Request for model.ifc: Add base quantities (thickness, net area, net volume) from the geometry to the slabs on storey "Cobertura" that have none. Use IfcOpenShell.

First a look at what the model holds.

```python
import ifcopenshell
import ifcopenshell.util.element
import ifcopenshell.util.unit

model = ifcopenshell.open("model.ifc")
print(model.schema)
for unit_type in ("LENGTHUNIT", "AREAUNIT", "VOLUMEUNIT"):
    print(unit_type, ifcopenshell.util.unit.calculate_unit_scale(model, unit_type))
storey = next(s for s in model.by_type("IfcBuildingStorey") if s.Name == "Cobertura")
slabs = [e for e in ifcopenshell.util.element.get_decomposition(storey) if e.is_a("IfcSlab")]
for e in sorted(slabs, key=lambda e: e.id()):
    print(e.id(), e.is_a(), e.Name, list(ifcopenshell.util.element.get_psets(e, qtos_only=True)), sep=" | ")
```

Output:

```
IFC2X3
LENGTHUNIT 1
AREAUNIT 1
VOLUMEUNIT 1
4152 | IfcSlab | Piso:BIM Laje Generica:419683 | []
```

```python
import ifcopenshell
import ifcopenshell.api.pset
import ifcopenshell.geom
import ifcopenshell.util.element
import ifcopenshell.util.shape
import ifcopenshell.util.unit

model = ifcopenshell.open("model.ifc")
unit_scale = ifcopenshell.util.unit.calculate_unit_scale(model)
area_scale = ifcopenshell.util.unit.calculate_unit_scale(model, "AREAUNIT")
volume_scale = ifcopenshell.util.unit.calculate_unit_scale(model, "VOLUMEUNIT")
settings = ifcopenshell.geom.settings()

storey = next(s for s in model.by_type("IfcBuildingStorey") if s.Name == "Cobertura")
slabs = [e for e in ifcopenshell.util.element.get_decomposition(storey) if e.is_a("IfcSlab")]

for e in sorted(slabs, key=lambda e: e.id()):
    if ifcopenshell.util.element.get_psets(e, qtos_only=True, should_inherit=False):
        continue
    # Geometry comes back in metres, in the element's own axes.
    shape = ifcopenshell.geom.create_shape(settings, e)
    values = {
        "Width": ifcopenshell.util.shape.get_z(shape.geometry) / unit_scale,
        "NetArea": ifcopenshell.util.shape.get_footprint_area(shape.geometry) / area_scale,
        "NetVolume": ifcopenshell.util.shape.get_volume(shape.geometry) / volume_scale,
    }
    qto = ifcopenshell.api.pset.add_qto(model, product=e, name="BaseQuantities")
    ifcopenshell.api.pset.edit_qto(model, qto=qto, properties=values)
    print(e.id(), {k: round(v, 3) for k, v in values.items()})

model.write("model_updated.ifc")
```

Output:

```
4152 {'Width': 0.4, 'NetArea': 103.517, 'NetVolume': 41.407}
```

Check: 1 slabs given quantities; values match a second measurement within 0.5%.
